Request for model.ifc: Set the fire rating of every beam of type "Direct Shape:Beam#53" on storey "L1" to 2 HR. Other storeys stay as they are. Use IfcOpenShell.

First a look at what the model holds.

```python
import ifcopenshell
import ifcopenshell.util.element

model = ifcopenshell.open("model.ifc")
print(model.schema)
storey = next(s for s in model.by_type("IfcBuildingStorey") if s.Name == "L1")
beams = [e for e in ifcopenshell.util.element.get_decomposition(storey) if e.is_a("IfcBeam")]
seen = {}
for e in beams:
    element_type = ifcopenshell.util.element.get_type(e)
    key = (element_type.Name if element_type != e and element_type else None, ifcopenshell.util.element.get_pset(e, "Pset_BeamCommon", "FireRating"))
    seen[key] = seen.get(key, 0) + 1
for (name, value), count in sorted(seen.items(), key=str):
    print(count, "x", name, "|", value)
```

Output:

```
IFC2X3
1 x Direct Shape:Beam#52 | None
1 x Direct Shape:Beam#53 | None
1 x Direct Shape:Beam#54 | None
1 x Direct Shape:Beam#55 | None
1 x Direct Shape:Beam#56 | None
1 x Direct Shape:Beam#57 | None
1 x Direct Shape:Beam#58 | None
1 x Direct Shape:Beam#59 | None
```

```python
import ifcopenshell
import ifcopenshell.api.pset
import ifcopenshell.util.element

model = ifcopenshell.open("model.ifc")

storey = next(s for s in model.by_type("IfcBuildingStorey") if s.Name == "L1")
beams = [e for e in ifcopenshell.util.element.get_decomposition(storey) if e.is_a("IfcBeam")]

count = 0
for e in beams:
    element_type = ifcopenshell.util.element.get_type(e)
    if element_type in (None, e) or element_type.Name != "Direct Shape:Beam#53":
        continue
    # add_pset returns the element's existing set when there is one.
    pset = ifcopenshell.api.pset.add_pset(model, product=e, name="Pset_BeamCommon")
    ifcopenshell.api.pset.edit_pset(model, pset=pset, properties={"FireRating": "2 HR"})
    count += 1

print(count, "beams updated")

model.write("model_v2.ifc")
```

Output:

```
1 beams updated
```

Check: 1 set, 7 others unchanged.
